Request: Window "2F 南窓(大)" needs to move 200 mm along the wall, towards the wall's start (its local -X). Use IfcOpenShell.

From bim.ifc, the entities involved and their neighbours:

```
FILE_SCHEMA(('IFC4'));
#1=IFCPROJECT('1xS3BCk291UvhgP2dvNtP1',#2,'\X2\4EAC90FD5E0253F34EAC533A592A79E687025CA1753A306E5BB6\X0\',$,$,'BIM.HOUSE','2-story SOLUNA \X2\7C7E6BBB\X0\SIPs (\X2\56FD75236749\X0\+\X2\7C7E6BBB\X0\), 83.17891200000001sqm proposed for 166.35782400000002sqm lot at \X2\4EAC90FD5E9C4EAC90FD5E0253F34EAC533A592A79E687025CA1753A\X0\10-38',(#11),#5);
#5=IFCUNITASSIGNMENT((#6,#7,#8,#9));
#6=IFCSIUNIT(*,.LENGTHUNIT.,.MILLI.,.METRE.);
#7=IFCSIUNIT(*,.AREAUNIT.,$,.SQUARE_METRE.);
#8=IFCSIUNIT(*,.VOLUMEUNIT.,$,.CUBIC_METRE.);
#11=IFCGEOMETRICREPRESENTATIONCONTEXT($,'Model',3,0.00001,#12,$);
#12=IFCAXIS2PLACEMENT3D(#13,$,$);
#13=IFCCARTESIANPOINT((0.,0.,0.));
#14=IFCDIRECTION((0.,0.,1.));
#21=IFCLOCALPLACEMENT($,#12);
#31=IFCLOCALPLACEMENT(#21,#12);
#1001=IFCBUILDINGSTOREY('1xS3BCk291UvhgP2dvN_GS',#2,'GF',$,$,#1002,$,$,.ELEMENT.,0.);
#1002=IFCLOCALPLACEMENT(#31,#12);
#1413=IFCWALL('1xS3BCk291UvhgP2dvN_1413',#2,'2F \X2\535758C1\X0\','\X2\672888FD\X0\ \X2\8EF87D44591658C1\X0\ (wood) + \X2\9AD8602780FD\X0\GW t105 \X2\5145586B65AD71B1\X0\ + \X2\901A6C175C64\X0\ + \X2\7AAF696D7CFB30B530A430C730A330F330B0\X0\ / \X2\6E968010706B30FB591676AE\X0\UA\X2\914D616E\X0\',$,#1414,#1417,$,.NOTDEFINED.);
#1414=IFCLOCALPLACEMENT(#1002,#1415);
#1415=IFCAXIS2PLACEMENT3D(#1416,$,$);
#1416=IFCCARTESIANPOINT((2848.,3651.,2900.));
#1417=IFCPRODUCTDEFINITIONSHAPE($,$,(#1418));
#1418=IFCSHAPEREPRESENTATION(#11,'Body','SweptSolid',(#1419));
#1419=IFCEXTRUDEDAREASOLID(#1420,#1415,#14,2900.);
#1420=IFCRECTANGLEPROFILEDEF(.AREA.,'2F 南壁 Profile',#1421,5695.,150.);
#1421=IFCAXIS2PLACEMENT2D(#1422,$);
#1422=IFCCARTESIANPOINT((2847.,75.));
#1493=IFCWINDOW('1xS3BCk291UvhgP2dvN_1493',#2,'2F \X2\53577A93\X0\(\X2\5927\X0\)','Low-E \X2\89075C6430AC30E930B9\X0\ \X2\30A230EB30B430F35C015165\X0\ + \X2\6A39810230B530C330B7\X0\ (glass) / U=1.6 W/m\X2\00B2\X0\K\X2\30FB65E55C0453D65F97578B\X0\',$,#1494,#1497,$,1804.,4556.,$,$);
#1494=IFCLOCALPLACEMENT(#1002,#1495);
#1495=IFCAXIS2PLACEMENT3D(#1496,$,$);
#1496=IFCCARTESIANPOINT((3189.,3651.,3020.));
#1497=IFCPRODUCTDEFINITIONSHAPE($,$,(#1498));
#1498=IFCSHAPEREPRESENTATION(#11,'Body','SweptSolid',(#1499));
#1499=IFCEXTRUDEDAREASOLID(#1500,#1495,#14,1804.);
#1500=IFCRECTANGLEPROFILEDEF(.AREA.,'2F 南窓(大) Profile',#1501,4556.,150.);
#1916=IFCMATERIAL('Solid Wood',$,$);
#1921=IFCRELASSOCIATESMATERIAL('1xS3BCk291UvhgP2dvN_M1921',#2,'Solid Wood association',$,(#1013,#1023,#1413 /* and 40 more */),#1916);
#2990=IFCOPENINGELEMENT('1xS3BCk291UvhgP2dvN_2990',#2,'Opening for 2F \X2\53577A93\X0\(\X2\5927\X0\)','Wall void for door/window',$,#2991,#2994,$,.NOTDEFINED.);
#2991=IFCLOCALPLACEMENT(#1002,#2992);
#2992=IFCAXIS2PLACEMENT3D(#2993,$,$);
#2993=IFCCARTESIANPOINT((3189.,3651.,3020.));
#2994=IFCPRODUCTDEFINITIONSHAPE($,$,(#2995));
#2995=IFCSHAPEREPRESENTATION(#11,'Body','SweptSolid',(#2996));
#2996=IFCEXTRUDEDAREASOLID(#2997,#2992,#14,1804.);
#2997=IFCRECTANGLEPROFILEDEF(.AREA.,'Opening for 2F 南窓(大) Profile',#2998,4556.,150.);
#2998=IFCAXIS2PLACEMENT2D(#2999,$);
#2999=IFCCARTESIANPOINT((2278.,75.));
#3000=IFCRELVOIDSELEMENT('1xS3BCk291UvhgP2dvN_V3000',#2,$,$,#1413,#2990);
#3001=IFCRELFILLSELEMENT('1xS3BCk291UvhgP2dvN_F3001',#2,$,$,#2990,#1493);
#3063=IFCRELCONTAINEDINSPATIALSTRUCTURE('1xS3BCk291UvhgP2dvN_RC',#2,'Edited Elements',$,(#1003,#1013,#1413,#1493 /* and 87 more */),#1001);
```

```python
import ifcopenshell
import ifcopenshell.api.geometry
import ifcopenshell.util.placement
import ifcopenshell.util.unit

model = ifcopenshell.open("bim.ifc")
unit_scale = ifcopenshell.util.unit.calculate_unit_scale(model)

window = model.by_id(1493)
opening = window.FillsVoids[0].RelatingOpeningElement
wall = opening.VoidsElements[0].RelatingBuildingElement

wall_matrix = ifcopenshell.util.placement.get_local_placement(wall.ObjectPlacement)
shift = wall_matrix[:3, 0] * -0.2 / unit_scale
before = ifcopenshell.util.placement.get_local_placement(window.ObjectPlacement)[:3, 3].copy()

# The window is not placed relative to its opening, so move both.
for product in (opening, window):
    matrix = ifcopenshell.util.placement.get_local_placement(product.ObjectPlacement)
    matrix[:3, 3] += shift
    ifcopenshell.api.geometry.edit_object_placement(model, product=product, matrix=matrix, is_si=False)

after = ifcopenshell.util.placement.get_local_placement(window.ObjectPlacement)[:3, 3]
print("window moved by", (after - before).round(3) + 0.0)

model.write("bim_v2.ifc")
```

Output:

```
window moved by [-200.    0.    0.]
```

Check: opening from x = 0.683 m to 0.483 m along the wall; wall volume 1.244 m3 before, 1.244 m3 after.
